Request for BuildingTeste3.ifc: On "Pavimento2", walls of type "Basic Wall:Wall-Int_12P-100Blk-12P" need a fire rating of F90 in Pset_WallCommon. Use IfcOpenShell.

First a look at what the model holds.

```python
import ifcopenshell
import ifcopenshell.util.element

model = ifcopenshell.open("BuildingTeste3.ifc")
print(model.schema)
storey = next(s for s in model.by_type("IfcBuildingStorey") if s.Name == "Pavimento2")
walls = [e for e in ifcopenshell.util.element.get_decomposition(storey) if e.is_a("IfcWall")]
seen = {}
for e in walls:
    element_type = ifcopenshell.util.element.get_type(e)
    key = (element_type.Name if element_type != e and element_type else None, ifcopenshell.util.element.get_pset(e, "Pset_WallCommon", "FireRating"))
    seen[key] = seen.get(key, 0) + 1
for (name, value), count in sorted(seen.items(), key=str):
    print(count, "x", name, "|", value)
```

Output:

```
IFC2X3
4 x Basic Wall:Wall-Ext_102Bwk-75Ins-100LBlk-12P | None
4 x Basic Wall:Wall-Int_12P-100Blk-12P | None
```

```python
import ifcopenshell
import ifcopenshell.api.pset
import ifcopenshell.util.element

model = ifcopenshell.open("BuildingTeste3.ifc")

storey = next(s for s in model.by_type("IfcBuildingStorey") if s.Name == "Pavimento2")
walls = [e for e in ifcopenshell.util.element.get_decomposition(storey) if e.is_a("IfcWall")]

count = 0
for e in walls:
    element_type = ifcopenshell.util.element.get_type(e)
    if element_type in (None, e) or element_type.Name != "Basic Wall:Wall-Int_12P-100Blk-12P":
        continue
    # add_pset returns the element's existing set when there is one.
    pset = ifcopenshell.api.pset.add_pset(model, product=e, name="Pset_WallCommon")
    ifcopenshell.api.pset.edit_pset(model, pset=pset, properties={"FireRating": "F90"})
    count += 1

print(count, "walls updated")

model.write("BuildingTeste3_updated.ifc")
```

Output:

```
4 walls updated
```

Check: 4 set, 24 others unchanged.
